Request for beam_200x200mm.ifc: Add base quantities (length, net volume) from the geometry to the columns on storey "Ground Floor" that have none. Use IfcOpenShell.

First a look at what the model holds.

```python
import ifcopenshell
import ifcopenshell.util.element
import ifcopenshell.util.unit

model = ifcopenshell.open("beam_200x200mm.ifc")
print(model.schema)
for unit_type in ("LENGTHUNIT", "AREAUNIT", "VOLUMEUNIT"):
    print(unit_type, ifcopenshell.util.unit.calculate_unit_scale(model, unit_type))
storey = next(s for s in model.by_type("IfcBuildingStorey") if s.Name == "Ground Floor")
columns = [e for e in ifcopenshell.util.element.get_decomposition(storey) if e.is_a("IfcColumn")]
for e in sorted(columns, key=lambda e: e.id()):
    print(e.id(), e.is_a(), e.Name, list(ifcopenshell.util.element.get_psets(e, qtos_only=True)), sep=" | ")
```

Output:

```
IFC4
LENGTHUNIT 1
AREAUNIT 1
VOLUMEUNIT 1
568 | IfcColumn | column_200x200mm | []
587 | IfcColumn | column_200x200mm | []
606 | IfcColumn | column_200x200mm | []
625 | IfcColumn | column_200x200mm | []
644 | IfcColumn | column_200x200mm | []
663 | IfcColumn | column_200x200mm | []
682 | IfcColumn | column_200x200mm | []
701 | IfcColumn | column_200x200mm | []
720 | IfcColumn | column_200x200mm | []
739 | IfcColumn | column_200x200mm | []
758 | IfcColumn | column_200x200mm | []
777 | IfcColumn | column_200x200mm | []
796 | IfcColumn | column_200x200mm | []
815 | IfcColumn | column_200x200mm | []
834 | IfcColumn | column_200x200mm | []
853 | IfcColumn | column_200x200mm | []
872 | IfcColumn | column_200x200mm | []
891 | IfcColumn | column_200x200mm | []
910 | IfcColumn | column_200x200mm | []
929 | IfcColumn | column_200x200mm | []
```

```python
import ifcopenshell
import ifcopenshell.api.pset
import ifcopenshell.geom
import ifcopenshell.util.element
import ifcopenshell.util.shape
import ifcopenshell.util.unit

model = ifcopenshell.open("beam_200x200mm.ifc")
unit_scale = ifcopenshell.util.unit.calculate_unit_scale(model)
volume_scale = ifcopenshell.util.unit.calculate_unit_scale(model, "VOLUMEUNIT")
settings = ifcopenshell.geom.settings()

storey = next(s for s in model.by_type("IfcBuildingStorey") if s.Name == "Ground Floor")
columns = [e for e in ifcopenshell.util.element.get_decomposition(storey) if e.is_a("IfcColumn")]

for e in sorted(columns, key=lambda e: e.id()):
    if ifcopenshell.util.element.get_psets(e, qtos_only=True, should_inherit=False):
        continue
    # Geometry comes back in metres, in the element's own axes.
    shape = ifcopenshell.geom.create_shape(settings, e)
    values = {
        "Length": ifcopenshell.util.shape.get_z(shape.geometry) / unit_scale,
        "NetVolume": ifcopenshell.util.shape.get_volume(shape.geometry) / volume_scale,
    }
    qto = ifcopenshell.api.pset.add_qto(model, product=e, name="Qto_ColumnBaseQuantities")
    ifcopenshell.api.pset.edit_qto(model, qto=qto, properties=values)
    print(e.id(), {k: round(v, 3) for k, v in values.items()})

model.write("beam_200x200mm-out.ifc")
```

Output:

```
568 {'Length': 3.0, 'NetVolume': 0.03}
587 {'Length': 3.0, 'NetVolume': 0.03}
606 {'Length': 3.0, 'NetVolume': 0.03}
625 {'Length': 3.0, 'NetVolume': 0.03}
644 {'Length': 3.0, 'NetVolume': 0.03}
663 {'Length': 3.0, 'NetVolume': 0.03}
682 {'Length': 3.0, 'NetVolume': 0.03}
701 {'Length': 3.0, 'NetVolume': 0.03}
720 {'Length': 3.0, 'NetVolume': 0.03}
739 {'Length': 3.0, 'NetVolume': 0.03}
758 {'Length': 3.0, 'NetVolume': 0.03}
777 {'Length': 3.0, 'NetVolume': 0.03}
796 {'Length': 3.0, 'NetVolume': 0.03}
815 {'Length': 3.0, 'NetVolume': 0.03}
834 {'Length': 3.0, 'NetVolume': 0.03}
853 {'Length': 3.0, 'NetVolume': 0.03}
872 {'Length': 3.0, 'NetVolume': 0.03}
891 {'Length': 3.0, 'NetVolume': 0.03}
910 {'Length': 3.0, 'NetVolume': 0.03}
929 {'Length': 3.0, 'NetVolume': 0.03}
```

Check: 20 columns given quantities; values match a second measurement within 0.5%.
